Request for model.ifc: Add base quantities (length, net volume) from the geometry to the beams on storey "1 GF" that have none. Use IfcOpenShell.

First a look at what the model holds.

```python
import ifcopenshell
import ifcopenshell.util.element
import ifcopenshell.util.unit

model = ifcopenshell.open("model.ifc")
print(model.schema)
for unit_type in ("LENGTHUNIT", "AREAUNIT", "VOLUMEUNIT"):
    print(unit_type, ifcopenshell.util.unit.calculate_unit_scale(model, unit_type))
storey = next(s for s in model.by_type("IfcBuildingStorey") if s.Name == "1 GF")
beams = [e for e in ifcopenshell.util.element.get_decomposition(storey) if e.is_a("IfcBeam")]
for e in sorted(beams, key=lambda e: e.id()):
    print(e.id(), e.is_a(), e.Name, list(ifcopenshell.util.element.get_psets(e, qtos_only=True)), sep=" | ")
```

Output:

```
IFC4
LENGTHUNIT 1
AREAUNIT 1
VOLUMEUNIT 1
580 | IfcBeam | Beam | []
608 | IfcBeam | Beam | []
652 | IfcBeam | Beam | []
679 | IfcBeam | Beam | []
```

```python
import ifcopenshell
import ifcopenshell.api.pset
import ifcopenshell.geom
import ifcopenshell.util.element
import ifcopenshell.util.shape
import ifcopenshell.util.unit

model = ifcopenshell.open("model.ifc")
unit_scale = ifcopenshell.util.unit.calculate_unit_scale(model)
volume_scale = ifcopenshell.util.unit.calculate_unit_scale(model, "VOLUMEUNIT")
settings = ifcopenshell.geom.settings()

storey = next(s for s in model.by_type("IfcBuildingStorey") if s.Name == "1 GF")
beams = [e for e in ifcopenshell.util.element.get_decomposition(storey) if e.is_a("IfcBeam")]

for e in sorted(beams, key=lambda e: e.id()):
    if ifcopenshell.util.element.get_psets(e, qtos_only=True, should_inherit=False):
        continue
    # Geometry comes back in metres, in the element's own axes.
    shape = ifcopenshell.geom.create_shape(settings, e)
    values = {
        "Length": ifcopenshell.util.shape.get_max_xyz(shape.geometry) / unit_scale,
        "NetVolume": ifcopenshell.util.shape.get_volume(shape.geometry) / volume_scale,
    }
    qto = ifcopenshell.api.pset.add_qto(model, product=e, name="Qto_BeamBaseQuantities")
    ifcopenshell.api.pset.edit_qto(model, qto=qto, properties=values)
    print(e.id(), {k: round(v, 3) for k, v in values.items()})

model.write("model-out.ifc")
```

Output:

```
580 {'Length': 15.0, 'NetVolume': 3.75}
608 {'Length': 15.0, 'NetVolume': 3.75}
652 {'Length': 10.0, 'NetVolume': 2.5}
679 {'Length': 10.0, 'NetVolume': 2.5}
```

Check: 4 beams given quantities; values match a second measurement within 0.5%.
